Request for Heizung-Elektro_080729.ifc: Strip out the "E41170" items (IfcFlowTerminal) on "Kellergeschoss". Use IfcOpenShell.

First a look at what the model holds.

```python
import ifcopenshell
import ifcopenshell.util.element

model = ifcopenshell.open("Heizung-Elektro_080729.ifc")
print(model.schema)
storey = next(s for s in model.by_type("IfcBuildingStorey") if s.Name == "Kellergeschoss")
terminals = [e for e in ifcopenshell.util.element.get_decomposition(storey) if e.is_a("IfcFlowTerminal")]
seen = {}
for e in terminals:
    element_type = ifcopenshell.util.element.get_type(e)
    name = element_type.Name if element_type not in (None, e) else None
    seen[name] = seen.get(name, 0) + 1
for name, count in sorted(seen.items(), key=str):
    print(count, "x", name)
```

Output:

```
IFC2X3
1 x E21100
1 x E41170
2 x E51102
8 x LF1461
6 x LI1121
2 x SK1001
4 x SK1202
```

```python
import ifcopenshell
import ifcopenshell.api.root
import ifcopenshell.util.element

model = ifcopenshell.open("Heizung-Elektro_080729.ifc")

storey = next(s for s in model.by_type("IfcBuildingStorey") if s.Name == "Kellergeschoss")
terminals = [e for e in ifcopenshell.util.element.get_decomposition(storey) if e.is_a("IfcFlowTerminal")]
targets = [e for e in terminals if (t := ifcopenshell.util.element.get_type(e)) not in (None, e) and t.Name == "E41170"]

for e in targets:
    ifcopenshell.api.root.remove_product(model, product=e)
print(len(targets), "removed")

model.write("Heizung-Elektro_080729-out.ifc")
```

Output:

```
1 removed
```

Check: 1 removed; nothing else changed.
